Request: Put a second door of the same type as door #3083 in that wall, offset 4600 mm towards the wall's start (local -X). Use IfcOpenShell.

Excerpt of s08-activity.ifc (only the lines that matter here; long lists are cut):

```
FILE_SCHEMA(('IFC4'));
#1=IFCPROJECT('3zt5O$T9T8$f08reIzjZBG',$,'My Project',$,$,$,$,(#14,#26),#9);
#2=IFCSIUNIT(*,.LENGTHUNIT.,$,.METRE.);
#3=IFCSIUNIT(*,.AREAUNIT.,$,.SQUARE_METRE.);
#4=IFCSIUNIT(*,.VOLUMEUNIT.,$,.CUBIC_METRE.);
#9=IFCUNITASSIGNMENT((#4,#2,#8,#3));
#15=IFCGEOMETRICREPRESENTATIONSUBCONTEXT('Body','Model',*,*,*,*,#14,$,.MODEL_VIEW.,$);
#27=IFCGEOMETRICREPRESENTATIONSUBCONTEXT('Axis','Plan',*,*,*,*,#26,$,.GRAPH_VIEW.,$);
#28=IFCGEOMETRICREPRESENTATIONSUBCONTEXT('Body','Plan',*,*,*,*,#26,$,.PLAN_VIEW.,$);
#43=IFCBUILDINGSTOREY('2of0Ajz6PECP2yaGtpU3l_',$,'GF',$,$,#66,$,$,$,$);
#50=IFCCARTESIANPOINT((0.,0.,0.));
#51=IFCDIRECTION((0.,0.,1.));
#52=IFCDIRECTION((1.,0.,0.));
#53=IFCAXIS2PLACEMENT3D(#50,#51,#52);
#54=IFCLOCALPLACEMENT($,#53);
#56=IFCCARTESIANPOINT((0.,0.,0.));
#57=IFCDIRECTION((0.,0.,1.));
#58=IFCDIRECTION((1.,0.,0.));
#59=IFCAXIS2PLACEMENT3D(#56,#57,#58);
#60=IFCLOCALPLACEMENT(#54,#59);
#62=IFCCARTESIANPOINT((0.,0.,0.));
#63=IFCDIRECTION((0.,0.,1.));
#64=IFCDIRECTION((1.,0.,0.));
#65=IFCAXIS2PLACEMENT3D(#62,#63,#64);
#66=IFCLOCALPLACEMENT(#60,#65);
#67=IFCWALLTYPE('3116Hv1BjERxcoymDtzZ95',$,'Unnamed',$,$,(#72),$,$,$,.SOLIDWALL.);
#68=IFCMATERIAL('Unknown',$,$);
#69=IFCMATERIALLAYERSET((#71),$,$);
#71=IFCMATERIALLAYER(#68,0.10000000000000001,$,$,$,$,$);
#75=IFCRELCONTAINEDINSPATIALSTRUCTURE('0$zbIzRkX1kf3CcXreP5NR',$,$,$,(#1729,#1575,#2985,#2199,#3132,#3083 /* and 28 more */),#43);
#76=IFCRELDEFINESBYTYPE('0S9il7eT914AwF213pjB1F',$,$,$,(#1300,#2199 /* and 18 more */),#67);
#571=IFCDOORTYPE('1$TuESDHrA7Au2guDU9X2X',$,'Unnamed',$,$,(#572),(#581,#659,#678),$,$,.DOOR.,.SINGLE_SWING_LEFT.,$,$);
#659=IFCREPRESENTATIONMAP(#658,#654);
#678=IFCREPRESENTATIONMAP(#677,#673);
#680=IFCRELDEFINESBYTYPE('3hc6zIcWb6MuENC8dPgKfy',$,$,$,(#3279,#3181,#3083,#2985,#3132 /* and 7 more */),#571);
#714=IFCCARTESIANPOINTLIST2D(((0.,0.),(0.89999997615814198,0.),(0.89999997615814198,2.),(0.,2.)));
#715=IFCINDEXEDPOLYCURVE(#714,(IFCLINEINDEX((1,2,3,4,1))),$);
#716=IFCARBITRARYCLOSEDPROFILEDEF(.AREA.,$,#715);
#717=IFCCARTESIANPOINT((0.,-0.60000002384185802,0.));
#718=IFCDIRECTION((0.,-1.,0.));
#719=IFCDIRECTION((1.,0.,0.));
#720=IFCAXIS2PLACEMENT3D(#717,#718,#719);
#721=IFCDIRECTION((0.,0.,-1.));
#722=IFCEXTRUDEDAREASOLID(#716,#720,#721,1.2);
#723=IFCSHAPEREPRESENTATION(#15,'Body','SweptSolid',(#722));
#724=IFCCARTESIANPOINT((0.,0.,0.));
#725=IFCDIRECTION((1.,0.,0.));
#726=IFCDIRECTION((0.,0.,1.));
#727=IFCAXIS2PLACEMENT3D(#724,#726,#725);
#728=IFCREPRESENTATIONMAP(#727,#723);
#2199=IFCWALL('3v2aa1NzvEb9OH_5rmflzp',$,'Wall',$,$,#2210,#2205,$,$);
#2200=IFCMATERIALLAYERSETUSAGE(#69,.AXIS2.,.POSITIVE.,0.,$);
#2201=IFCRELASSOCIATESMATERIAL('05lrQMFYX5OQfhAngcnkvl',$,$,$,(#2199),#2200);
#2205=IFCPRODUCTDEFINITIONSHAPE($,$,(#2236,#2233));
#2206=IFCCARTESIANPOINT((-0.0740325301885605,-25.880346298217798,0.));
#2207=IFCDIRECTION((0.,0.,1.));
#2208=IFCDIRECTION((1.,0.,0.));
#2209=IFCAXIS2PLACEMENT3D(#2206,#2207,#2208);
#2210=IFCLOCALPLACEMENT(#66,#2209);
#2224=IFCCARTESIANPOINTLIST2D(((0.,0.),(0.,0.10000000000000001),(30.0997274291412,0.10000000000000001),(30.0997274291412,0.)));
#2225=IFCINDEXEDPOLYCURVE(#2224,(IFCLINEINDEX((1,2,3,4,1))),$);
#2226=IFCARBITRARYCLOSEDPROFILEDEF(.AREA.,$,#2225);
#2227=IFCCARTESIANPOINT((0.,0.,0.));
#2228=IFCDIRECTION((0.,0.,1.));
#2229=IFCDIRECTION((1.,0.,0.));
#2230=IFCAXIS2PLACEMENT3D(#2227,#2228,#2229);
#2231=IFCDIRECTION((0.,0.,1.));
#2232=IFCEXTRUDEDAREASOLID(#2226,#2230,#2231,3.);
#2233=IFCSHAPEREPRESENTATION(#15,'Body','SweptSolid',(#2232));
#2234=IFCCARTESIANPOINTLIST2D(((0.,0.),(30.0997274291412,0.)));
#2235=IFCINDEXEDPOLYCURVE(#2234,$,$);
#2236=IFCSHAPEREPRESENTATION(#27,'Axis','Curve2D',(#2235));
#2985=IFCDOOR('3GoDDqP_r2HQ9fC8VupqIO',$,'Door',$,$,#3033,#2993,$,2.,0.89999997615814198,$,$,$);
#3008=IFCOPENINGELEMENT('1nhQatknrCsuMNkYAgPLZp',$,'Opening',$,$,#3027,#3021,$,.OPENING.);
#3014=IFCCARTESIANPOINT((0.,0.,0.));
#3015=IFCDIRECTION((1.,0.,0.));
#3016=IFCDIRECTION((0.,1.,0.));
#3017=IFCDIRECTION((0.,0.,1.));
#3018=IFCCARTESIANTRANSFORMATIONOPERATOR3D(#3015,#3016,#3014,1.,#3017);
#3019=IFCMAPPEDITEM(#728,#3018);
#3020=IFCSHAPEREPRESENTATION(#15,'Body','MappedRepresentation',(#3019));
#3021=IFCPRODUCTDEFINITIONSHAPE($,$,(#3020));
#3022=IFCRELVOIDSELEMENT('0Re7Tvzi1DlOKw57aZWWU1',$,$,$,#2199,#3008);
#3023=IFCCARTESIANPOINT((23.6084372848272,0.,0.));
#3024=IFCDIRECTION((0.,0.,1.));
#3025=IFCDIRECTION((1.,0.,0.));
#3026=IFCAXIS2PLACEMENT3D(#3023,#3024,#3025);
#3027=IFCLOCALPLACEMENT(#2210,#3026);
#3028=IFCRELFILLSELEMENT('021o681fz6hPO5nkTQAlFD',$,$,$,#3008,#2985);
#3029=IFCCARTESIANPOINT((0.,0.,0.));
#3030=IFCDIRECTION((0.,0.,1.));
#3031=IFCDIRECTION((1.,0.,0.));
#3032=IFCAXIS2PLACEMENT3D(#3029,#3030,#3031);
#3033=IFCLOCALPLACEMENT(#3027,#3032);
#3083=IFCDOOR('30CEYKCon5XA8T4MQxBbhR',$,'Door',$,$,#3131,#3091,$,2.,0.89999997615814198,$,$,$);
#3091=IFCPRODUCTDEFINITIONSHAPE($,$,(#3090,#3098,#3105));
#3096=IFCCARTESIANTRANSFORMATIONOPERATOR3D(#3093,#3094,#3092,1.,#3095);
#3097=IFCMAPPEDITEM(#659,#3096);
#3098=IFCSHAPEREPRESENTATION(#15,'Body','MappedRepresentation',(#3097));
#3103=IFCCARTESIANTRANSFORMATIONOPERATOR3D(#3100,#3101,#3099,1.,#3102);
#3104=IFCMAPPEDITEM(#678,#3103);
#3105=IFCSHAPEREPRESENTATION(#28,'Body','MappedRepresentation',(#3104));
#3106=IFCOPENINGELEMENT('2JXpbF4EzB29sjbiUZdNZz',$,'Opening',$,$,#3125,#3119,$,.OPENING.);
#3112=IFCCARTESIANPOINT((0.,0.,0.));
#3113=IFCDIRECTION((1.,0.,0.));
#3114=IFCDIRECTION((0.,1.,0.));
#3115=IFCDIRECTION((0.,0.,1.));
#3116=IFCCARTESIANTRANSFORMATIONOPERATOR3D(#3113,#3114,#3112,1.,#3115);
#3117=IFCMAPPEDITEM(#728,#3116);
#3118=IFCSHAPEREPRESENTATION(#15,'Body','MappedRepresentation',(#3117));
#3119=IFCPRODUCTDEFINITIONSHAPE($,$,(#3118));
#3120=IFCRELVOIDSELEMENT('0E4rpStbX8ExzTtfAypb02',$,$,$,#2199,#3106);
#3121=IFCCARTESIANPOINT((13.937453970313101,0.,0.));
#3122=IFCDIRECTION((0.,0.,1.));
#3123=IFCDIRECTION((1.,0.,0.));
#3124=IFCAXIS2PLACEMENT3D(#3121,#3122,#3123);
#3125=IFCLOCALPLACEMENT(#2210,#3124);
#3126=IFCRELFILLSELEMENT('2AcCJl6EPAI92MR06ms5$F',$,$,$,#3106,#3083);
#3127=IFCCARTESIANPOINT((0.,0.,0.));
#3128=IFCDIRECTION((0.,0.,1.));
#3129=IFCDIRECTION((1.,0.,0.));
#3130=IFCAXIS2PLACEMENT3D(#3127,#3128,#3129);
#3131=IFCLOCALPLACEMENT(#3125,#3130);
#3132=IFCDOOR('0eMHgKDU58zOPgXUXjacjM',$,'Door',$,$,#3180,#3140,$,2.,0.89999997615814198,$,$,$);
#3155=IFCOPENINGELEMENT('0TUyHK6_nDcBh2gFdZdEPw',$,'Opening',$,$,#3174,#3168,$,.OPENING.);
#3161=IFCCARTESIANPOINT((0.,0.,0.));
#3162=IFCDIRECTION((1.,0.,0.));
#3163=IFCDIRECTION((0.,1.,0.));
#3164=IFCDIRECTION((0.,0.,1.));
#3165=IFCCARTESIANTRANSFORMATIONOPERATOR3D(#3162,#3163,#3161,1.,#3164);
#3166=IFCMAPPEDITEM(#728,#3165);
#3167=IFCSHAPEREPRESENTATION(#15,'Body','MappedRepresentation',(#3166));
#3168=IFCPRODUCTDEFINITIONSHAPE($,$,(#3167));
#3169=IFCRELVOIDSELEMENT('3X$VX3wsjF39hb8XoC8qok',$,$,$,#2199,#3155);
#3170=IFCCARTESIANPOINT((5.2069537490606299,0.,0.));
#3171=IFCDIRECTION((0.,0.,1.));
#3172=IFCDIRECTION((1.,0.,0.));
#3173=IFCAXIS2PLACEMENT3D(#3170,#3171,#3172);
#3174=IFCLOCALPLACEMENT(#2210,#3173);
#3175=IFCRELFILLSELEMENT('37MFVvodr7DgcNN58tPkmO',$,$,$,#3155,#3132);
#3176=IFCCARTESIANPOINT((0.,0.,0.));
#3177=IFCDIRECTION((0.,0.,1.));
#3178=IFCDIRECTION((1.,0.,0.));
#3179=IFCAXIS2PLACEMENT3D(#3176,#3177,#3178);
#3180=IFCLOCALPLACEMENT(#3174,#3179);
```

```python
import ifcopenshell
import ifcopenshell.api.feature
import ifcopenshell.api.geometry
import ifcopenshell.api.root
import ifcopenshell.geom
import ifcopenshell.util.element
import ifcopenshell.util.placement
import ifcopenshell.util.shape

model = ifcopenshell.open("s08-activity.ifc")
settings = ifcopenshell.geom.settings()


def volume(element):
    """Net volume in cubic metres, openings subtracted."""
    shape = ifcopenshell.geom.create_shape(settings, element)
    return ifcopenshell.util.shape.get_volume(shape.geometry)


door = model.by_guid("30CEYKCon5XA8T4MQxBbhR")
opening = door.FillsVoids[0].RelatingOpeningElement
wall = opening.VoidsElements[0].RelatingBuildingElement
before = volume(wall)
shift = ifcopenshell.util.placement.get_local_placement(wall.ObjectPlacement)[:3, 0] * -4.6

# copy_class copies the void relationship, type, container and properties, but no geometry.
new_opening = ifcopenshell.api.root.copy_class(model, product=opening)
new_opening.Representation = ifcopenshell.util.element.copy_deep(
    model, opening.Representation, exclude=["IfcGeometricRepresentationContext", "IfcRepresentationMap"]
)
new_door = ifcopenshell.api.root.copy_class(model, product=door)
new_door.Representation = ifcopenshell.util.element.copy_deep(
    model, door.Representation, exclude=["IfcGeometricRepresentationContext", "IfcRepresentationMap"]
)
ifcopenshell.api.feature.add_filling(model, opening=new_opening, element=new_door)

for old, new in ((opening, new_opening), (door, new_door)):
    matrix = ifcopenshell.util.placement.get_local_placement(old.ObjectPlacement)
    matrix[:3, 3] += shift
    ifcopenshell.api.geometry.edit_object_placement(model, product=new, matrix=matrix, is_si=False)

after = volume(wall)

print(f"wall volume {before:.3f} -> {after:.3f} m3")

model.write("s08-activity_updated.ifc")
```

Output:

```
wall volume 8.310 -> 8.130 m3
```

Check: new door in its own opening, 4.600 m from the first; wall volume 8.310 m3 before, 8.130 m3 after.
